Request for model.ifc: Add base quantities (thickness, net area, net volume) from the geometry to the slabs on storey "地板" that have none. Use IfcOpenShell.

First a look at what the model holds.

```python
import ifcopenshell
import ifcopenshell.util.element
import ifcopenshell.util.unit

model = ifcopenshell.open("model.ifc")
print(model.schema)
for unit_type in ("LENGTHUNIT", "AREAUNIT", "VOLUMEUNIT"):
    print(unit_type, ifcopenshell.util.unit.calculate_unit_scale(model, unit_type))
storey = next(s for s in model.by_type("IfcBuildingStorey") if s.Name == "地板")
slabs = [e for e in ifcopenshell.util.element.get_decomposition(storey) if e.is_a("IfcSlab")]
for e in sorted(slabs, key=lambda e: e.id()):
    print(e.id(), e.is_a(), e.Name, list(ifcopenshell.util.element.get_psets(e, qtos_only=True)), sep=" | ")
```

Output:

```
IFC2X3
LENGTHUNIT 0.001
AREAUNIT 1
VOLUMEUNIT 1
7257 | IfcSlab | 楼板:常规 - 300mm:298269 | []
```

```python
import ifcopenshell
import ifcopenshell.api.pset
import ifcopenshell.geom
import ifcopenshell.util.element
import ifcopenshell.util.shape
import ifcopenshell.util.unit

model = ifcopenshell.open("model.ifc")
unit_scale = ifcopenshell.util.unit.calculate_unit_scale(model)
area_scale = ifcopenshell.util.unit.calculate_unit_scale(model, "AREAUNIT")
volume_scale = ifcopenshell.util.unit.calculate_unit_scale(model, "VOLUMEUNIT")
settings = ifcopenshell.geom.settings()

storey = next(s for s in model.by_type("IfcBuildingStorey") if s.Name == "地板")
slabs = [e for e in ifcopenshell.util.element.get_decomposition(storey) if e.is_a("IfcSlab")]

for e in sorted(slabs, key=lambda e: e.id()):
    if ifcopenshell.util.element.get_psets(e, qtos_only=True, should_inherit=False):
        continue
    # Geometry comes back in metres, in the element's own axes.
    shape = ifcopenshell.geom.create_shape(settings, e)
    values = {
        "Width": ifcopenshell.util.shape.get_z(shape.geometry) / unit_scale,
        "NetArea": ifcopenshell.util.shape.get_footprint_area(shape.geometry) / area_scale,
        "NetVolume": ifcopenshell.util.shape.get_volume(shape.geometry) / volume_scale,
    }
    qto = ifcopenshell.api.pset.add_qto(model, product=e, name="BaseQuantities")
    ifcopenshell.api.pset.edit_qto(model, qto=qto, properties=values)
    print(e.id(), {k: round(v, 3) for k, v in values.items()})

model.write("model_updated.ifc")
```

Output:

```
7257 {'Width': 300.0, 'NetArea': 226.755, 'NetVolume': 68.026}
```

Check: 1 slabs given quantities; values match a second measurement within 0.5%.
